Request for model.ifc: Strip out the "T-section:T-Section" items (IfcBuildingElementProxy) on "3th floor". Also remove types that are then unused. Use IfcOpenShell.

First a look at what the model holds.

```python
import ifcopenshell
import ifcopenshell.util.element

model = ifcopenshell.open("model.ifc")
print(model.schema)
storey = next(s for s in model.by_type("IfcBuildingStorey") if s.Name == "3th floor")
proxies = [e for e in ifcopenshell.util.element.get_decomposition(storey) if e.is_a("IfcBuildingElementProxy")]
seen = {}
for e in proxies:
    element_type = ifcopenshell.util.element.get_type(e)
    name = element_type.Name if element_type not in (None, e) else None
    seen[name] = seen.get(name, 0) + 1
for name, count in sorted(seen.items(), key=str):
    print(count, "x", name)
```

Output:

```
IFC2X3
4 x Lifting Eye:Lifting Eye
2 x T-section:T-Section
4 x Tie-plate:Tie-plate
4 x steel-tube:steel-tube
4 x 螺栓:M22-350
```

```python
import ifcopenshell
import ifcopenshell.api.root
import ifcopenshell.util.element

model = ifcopenshell.open("model.ifc")

storey = next(s for s in model.by_type("IfcBuildingStorey") if s.Name == "3th floor")
proxies = [e for e in ifcopenshell.util.element.get_decomposition(storey) if e.is_a("IfcBuildingElementProxy")]
targets = [e for e in proxies if (t := ifcopenshell.util.element.get_type(e)) not in (None, e) and t.Name == "T-section:T-Section"]
types = {ifcopenshell.util.element.get_type(e) for e in targets} - {None, *targets}

for e in targets:
    ifcopenshell.api.root.remove_product(model, product=e)
print(len(targets), "removed")

unused = [t for t in types if not ifcopenshell.util.element.get_types(t)]
for t in unused:
    ifcopenshell.api.root.remove_product(model, product=t)
print(len(unused), "unused types removed")

model.write("model_updated.ifc")
```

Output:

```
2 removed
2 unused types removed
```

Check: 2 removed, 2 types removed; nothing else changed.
